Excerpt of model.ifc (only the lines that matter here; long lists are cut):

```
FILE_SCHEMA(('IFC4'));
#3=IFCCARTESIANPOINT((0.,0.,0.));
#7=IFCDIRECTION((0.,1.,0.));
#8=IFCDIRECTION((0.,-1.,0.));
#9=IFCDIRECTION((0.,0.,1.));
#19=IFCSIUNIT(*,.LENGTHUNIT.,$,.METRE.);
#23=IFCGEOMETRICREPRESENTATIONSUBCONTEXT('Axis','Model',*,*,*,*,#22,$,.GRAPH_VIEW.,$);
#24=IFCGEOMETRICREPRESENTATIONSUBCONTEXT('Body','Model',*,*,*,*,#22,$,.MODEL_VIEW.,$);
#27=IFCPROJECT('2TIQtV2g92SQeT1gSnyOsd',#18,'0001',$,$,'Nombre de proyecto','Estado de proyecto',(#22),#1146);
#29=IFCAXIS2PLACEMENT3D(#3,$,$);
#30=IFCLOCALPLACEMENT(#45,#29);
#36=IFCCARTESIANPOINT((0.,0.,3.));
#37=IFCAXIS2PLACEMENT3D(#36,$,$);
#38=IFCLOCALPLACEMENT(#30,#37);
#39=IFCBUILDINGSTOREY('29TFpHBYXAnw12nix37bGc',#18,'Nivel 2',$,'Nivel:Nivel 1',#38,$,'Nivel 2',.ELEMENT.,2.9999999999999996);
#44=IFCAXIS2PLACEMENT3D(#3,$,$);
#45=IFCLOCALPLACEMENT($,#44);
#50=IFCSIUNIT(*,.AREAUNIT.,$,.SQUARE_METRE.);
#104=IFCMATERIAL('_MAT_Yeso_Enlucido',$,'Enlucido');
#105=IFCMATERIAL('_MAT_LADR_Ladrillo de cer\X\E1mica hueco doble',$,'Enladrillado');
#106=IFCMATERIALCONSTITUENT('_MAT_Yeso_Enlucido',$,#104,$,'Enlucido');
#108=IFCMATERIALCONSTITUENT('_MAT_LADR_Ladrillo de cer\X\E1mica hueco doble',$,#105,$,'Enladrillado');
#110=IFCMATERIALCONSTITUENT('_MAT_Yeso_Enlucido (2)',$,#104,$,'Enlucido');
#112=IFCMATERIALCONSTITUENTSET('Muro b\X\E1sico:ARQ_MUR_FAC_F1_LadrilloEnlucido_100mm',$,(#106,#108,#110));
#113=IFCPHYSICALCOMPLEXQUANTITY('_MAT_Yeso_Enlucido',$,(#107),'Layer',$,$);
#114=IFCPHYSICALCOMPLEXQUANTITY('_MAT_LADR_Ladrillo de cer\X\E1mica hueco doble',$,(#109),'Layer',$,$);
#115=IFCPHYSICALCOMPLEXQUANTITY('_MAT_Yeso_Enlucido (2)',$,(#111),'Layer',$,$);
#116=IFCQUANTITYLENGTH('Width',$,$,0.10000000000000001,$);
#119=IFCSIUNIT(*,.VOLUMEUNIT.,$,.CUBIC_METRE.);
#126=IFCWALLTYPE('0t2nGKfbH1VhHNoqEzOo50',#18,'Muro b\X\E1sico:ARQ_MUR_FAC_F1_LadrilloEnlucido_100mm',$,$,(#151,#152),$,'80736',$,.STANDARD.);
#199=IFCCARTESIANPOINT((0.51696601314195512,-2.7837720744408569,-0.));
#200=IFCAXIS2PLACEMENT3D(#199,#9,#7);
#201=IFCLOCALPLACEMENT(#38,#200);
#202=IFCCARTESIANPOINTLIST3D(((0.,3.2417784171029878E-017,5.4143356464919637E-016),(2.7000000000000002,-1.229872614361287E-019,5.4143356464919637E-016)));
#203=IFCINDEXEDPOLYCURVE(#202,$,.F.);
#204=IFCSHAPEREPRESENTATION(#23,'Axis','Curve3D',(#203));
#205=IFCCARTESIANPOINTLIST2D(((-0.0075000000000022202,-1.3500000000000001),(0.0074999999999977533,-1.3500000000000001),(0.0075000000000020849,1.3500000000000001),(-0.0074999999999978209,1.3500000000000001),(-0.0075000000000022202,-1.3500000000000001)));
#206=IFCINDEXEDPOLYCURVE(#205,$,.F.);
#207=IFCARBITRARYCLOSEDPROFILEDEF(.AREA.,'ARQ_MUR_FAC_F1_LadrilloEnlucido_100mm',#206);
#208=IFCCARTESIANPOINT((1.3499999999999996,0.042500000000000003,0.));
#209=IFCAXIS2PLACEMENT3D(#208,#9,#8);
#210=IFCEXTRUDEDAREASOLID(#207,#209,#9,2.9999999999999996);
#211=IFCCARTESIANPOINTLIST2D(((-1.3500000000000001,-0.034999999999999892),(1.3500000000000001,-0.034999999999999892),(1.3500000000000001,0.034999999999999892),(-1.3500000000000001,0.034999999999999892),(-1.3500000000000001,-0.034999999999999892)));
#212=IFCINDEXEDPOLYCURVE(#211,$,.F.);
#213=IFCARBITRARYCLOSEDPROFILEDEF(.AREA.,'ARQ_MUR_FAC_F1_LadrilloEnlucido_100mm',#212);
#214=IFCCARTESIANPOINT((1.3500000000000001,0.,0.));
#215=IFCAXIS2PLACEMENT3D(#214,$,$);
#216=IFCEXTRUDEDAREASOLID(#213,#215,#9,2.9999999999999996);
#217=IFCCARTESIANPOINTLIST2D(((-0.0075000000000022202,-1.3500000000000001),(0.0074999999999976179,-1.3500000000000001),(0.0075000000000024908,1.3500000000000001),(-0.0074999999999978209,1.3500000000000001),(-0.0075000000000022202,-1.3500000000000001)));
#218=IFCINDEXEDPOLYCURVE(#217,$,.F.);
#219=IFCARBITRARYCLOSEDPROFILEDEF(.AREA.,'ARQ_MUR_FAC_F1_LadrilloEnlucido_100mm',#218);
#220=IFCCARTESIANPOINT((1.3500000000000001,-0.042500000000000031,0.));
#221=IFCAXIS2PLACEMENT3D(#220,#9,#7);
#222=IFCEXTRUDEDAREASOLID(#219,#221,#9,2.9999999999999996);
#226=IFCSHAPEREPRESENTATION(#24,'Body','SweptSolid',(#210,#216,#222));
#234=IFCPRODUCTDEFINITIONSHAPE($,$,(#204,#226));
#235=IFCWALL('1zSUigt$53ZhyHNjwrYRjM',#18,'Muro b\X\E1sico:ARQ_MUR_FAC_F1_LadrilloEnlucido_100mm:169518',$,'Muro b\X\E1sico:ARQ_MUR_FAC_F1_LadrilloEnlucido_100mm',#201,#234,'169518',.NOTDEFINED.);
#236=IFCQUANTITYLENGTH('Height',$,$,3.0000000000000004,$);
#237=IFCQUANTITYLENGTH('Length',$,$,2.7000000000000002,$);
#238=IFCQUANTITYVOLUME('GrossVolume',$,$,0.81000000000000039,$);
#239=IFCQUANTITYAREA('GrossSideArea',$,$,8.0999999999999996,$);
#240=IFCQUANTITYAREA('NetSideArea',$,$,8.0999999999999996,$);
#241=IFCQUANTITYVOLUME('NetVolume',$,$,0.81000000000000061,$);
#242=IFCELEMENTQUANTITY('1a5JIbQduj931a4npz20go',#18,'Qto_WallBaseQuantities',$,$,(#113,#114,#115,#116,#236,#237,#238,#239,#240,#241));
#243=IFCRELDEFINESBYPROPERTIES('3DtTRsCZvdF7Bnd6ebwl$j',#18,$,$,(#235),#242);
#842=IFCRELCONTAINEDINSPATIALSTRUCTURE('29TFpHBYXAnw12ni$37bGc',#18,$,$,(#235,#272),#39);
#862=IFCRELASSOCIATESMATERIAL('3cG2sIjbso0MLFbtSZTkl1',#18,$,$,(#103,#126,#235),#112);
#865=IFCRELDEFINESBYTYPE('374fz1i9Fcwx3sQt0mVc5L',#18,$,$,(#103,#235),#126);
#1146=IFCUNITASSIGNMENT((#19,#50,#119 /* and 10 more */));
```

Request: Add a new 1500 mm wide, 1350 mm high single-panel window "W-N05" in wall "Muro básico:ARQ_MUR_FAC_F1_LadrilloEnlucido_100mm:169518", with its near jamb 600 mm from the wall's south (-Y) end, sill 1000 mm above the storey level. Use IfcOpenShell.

```python
import numpy as np
import ifcopenshell
import ifcopenshell.api.feature
import ifcopenshell.api.geometry
import ifcopenshell.api.pset
import ifcopenshell.api.root
import ifcopenshell.api.spatial
import ifcopenshell.geom
import ifcopenshell.util.element
import ifcopenshell.util.placement
import ifcopenshell.util.representation
import ifcopenshell.util.shape
import ifcopenshell.util.unit

model = ifcopenshell.open("model.ifc")
unit_scale = ifcopenshell.util.unit.calculate_unit_scale(model)
area_scale = ifcopenshell.util.unit.calculate_unit_scale(model, "AREAUNIT")
volume_scale = ifcopenshell.util.unit.calculate_unit_scale(model, "VOLUMEUNIT")
settings = ifcopenshell.geom.settings()


def volume(element):
    """Net volume in cubic metres, openings subtracted."""
    shape = ifcopenshell.geom.create_shape(settings, element)
    return ifcopenshell.util.shape.get_volume(shape.geometry)


wall = model.by_guid("1zSUigt$53ZhyHNjwrYRjM")
storey = ifcopenshell.util.element.get_container(wall, ifc_class="IfcBuildingStorey")
context = ifcopenshell.util.representation.get_context(model, "Model", "Body", "MODEL_VIEW")
before = volume(wall)

width, height, from_end, sill = 1.5, 1.35, 0.6, 1  # metres

# The wall runs along its own X axis, and the end named is its -X end.
wall_shape = ifcopenshell.geom.create_shape(settings, wall)
x, y, z = ifcopenshell.util.shape.get_vertices(wall_shape.geometry).T
start = x.min() + from_end
face, thickness = float(y.min()), float(y.max() - y.min())
wall_matrix = ifcopenshell.util.placement.get_local_placement(wall.ObjectPlacement)
level = ifcopenshell.util.placement.get_local_placement(storey.ObjectPlacement)[2, 3]


def in_wall(x, y):
    """Placement at x, y metres in the wall's axes, at sill height."""
    matrix = wall_matrix.copy()
    matrix[:, 3] = wall_matrix @ np.array([x / unit_scale, y / unit_scale, 0.0, 1.0])
    matrix[2, 3] = level + sill / unit_scale
    return matrix


# Opening: a box that overshoots both wall faces by 50 mm.
opening = ifcopenshell.api.root.create_entity(model, ifc_class="IfcOpeningElement", predefined_type="OPENING")
box = ifcopenshell.api.geometry.add_wall_representation(
    model, context=context, length=width, height=height, thickness=thickness + 0.1
)
ifcopenshell.api.geometry.assign_representation(model, product=opening, representation=box)
ifcopenshell.api.geometry.edit_object_placement(model, product=opening, matrix=in_wall(start, face - 0.05), is_si=False)
ifcopenshell.api.feature.add_feature(model, feature=opening, element=wall)

window = ifcopenshell.api.root.create_entity(model, ifc_class="IfcWindow", name="W-N05", predefined_type="WINDOW")
window.OverallWidth, window.OverallHeight = width / unit_scale, height / unit_scale
window.PartitioningType = "SINGLE_PANEL"
body = ifcopenshell.api.geometry.add_window_representation(
    model,
    context=context,
    overall_width=window.OverallWidth,
    overall_height=window.OverallHeight,
    partition_type="SINGLE_PANEL",
)
ifcopenshell.api.geometry.assign_representation(model, product=window, representation=body)
ifcopenshell.api.spatial.assign_container(model, products=[window], relating_structure=storey)
ifcopenshell.api.feature.add_filling(model, opening=opening, element=window)

# Centre the window in the wall's thickness.
ifcopenshell.api.geometry.edit_object_placement(model, product=window, matrix=in_wall(start, face), is_si=False)
window_shape = ifcopenshell.geom.create_shape(settings, window)
depth = ifcopenshell.util.shape.get_vertices(window_shape.geometry)[:, 1]
offset = face + thickness / 2 - (depth.min() + depth.max()) / 2
ifcopenshell.api.geometry.edit_object_placement(model, product=window, matrix=in_wall(start, offset), is_si=False)

after = volume(wall)

# Update the wall's stored quantities.
qto = model.by_id(ifcopenshell.util.element.get_pset(wall, "Qto_WallBaseQuantities", should_inherit=False)["id"])
ifcopenshell.api.pset.edit_qto(model, qto=qto, properties={
    "NetSideArea": after / thickness / area_scale,
    "NetVolume": after / volume_scale,
})

print(f"wall volume {before:.3f} -> {after:.3f} m3")

model.write("model-out.ifc")
```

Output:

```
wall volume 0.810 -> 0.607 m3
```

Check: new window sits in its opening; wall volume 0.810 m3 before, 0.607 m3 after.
